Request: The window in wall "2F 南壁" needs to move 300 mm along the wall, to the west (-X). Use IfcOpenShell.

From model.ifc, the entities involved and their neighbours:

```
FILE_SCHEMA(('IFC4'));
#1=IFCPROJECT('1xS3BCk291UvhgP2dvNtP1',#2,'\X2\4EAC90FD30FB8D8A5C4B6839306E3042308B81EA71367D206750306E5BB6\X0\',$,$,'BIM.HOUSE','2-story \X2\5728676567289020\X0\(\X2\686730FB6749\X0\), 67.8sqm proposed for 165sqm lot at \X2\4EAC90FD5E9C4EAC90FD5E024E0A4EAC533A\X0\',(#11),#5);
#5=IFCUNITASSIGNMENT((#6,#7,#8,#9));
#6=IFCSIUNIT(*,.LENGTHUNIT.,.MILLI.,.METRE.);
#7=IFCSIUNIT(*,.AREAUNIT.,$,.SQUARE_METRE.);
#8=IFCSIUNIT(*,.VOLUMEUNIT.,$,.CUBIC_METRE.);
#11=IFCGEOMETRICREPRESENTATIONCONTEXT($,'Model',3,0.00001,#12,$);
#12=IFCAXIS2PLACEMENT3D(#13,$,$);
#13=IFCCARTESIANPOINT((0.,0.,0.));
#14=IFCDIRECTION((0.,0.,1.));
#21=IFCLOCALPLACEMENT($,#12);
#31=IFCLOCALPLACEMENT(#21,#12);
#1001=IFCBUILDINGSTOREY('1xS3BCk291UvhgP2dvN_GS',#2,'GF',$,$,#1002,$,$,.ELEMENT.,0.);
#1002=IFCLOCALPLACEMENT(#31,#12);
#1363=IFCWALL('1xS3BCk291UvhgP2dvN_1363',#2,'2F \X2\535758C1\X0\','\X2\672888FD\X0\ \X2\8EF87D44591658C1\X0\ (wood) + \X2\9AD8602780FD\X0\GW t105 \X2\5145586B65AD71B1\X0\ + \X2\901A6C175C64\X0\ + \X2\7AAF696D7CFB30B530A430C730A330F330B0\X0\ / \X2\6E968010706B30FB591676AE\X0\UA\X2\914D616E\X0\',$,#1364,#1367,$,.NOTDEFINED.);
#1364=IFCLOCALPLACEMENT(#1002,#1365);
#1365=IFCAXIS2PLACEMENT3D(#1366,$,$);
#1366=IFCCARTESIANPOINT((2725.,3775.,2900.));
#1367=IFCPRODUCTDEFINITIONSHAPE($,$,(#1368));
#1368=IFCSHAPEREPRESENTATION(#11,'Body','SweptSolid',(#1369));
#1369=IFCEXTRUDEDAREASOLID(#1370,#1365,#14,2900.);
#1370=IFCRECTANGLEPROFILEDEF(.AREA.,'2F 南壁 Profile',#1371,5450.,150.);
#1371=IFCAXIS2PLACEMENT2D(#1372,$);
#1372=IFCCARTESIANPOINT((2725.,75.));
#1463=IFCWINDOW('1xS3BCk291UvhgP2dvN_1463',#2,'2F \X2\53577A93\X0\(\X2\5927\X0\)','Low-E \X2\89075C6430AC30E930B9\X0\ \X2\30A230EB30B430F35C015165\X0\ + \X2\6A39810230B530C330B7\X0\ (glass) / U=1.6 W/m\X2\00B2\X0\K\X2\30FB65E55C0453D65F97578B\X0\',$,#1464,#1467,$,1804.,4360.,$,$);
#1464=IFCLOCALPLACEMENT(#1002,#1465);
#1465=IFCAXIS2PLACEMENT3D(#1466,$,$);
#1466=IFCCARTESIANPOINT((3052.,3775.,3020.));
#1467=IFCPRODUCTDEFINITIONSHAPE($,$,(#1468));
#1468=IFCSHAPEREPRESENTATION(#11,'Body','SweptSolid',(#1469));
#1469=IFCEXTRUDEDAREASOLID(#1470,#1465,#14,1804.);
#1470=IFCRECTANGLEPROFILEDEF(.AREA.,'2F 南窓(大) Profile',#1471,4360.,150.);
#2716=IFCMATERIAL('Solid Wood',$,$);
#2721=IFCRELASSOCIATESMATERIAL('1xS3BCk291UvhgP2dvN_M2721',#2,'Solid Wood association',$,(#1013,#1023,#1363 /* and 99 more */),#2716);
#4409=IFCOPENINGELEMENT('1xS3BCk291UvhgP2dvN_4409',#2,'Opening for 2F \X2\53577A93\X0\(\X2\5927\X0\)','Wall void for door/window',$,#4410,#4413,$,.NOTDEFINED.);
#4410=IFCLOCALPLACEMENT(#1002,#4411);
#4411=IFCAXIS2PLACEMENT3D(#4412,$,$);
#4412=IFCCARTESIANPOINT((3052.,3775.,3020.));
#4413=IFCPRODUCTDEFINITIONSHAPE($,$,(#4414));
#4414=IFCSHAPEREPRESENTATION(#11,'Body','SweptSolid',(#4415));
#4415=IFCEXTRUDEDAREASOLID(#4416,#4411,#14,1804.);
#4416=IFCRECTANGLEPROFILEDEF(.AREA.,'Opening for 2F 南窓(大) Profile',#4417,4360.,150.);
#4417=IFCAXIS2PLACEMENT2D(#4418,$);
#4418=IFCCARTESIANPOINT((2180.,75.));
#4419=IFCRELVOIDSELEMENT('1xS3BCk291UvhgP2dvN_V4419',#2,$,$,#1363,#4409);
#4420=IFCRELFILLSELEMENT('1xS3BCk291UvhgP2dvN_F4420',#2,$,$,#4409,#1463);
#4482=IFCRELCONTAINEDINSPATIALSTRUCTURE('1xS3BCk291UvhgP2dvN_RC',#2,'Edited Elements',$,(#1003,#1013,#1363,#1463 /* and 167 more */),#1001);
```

```python
import ifcopenshell
import ifcopenshell.api.geometry
import ifcopenshell.util.placement
import ifcopenshell.util.unit

model = ifcopenshell.open("model.ifc")
unit_scale = ifcopenshell.util.unit.calculate_unit_scale(model)

window = model.by_guid("1xS3BCk291UvhgP2dvN_1463")
opening = window.FillsVoids[0].RelatingOpeningElement
wall = opening.VoidsElements[0].RelatingBuildingElement

wall_matrix = ifcopenshell.util.placement.get_local_placement(wall.ObjectPlacement)
shift = wall_matrix[:3, 0] * -0.3 / unit_scale
before = ifcopenshell.util.placement.get_local_placement(window.ObjectPlacement)[:3, 3].copy()

# The window is not placed relative to its opening, so move both.
for product in (opening, window):
    matrix = ifcopenshell.util.placement.get_local_placement(product.ObjectPlacement)
    matrix[:3, 3] += shift
    ifcopenshell.api.geometry.edit_object_placement(model, product=product, matrix=matrix, is_si=False)

after = ifcopenshell.util.placement.get_local_placement(window.ObjectPlacement)[:3, 3]
print("window moved by", (after - before).round(3) + 0.0)

model.write("model_rev.ifc")
```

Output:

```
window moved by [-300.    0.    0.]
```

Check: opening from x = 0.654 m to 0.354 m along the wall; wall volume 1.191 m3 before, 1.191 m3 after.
